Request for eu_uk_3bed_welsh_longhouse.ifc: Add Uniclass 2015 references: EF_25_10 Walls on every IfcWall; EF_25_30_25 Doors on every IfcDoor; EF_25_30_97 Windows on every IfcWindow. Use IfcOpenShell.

First a look at what the model holds.

```python
import ifcopenshell

model = ifcopenshell.open("eu_uk_3bed_welsh_longhouse.ifc")
print(model.schema)
print("classifications:", [c.Name for c in model.by_type("IfcClassification")])
for ifc_class in ("IfcDoor", "IfcRoof", "IfcStair", "IfcWall", "IfcWindow"):
    print(ifc_class, len(model.by_type(ifc_class)))
```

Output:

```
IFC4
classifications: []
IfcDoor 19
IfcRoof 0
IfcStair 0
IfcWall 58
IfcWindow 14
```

```python
import ifcopenshell
import ifcopenshell.api.classification

model = ifcopenshell.open("eu_uk_3bed_welsh_longhouse.ifc")

system = ifcopenshell.api.classification.add_classification(model, classification="Uniclass 2015")

codes = {
    "IfcWall": ("EF_25_10", "Walls"),
    "IfcDoor": ("EF_25_30_25", "Doors"),
    "IfcWindow": ("EF_25_30_97", "Windows"),
}
for ifc_class, (code, name) in codes.items():
    products = model.by_type(ifc_class)
    ifcopenshell.api.classification.add_reference(
        model, products=products, classification=system, identification=code, name=name
    )
    print(code, len(products))

model.write("eu_uk_3bed_welsh_longhouse_v2.ifc")
```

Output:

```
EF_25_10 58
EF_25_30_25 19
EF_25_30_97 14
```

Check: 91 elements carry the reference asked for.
